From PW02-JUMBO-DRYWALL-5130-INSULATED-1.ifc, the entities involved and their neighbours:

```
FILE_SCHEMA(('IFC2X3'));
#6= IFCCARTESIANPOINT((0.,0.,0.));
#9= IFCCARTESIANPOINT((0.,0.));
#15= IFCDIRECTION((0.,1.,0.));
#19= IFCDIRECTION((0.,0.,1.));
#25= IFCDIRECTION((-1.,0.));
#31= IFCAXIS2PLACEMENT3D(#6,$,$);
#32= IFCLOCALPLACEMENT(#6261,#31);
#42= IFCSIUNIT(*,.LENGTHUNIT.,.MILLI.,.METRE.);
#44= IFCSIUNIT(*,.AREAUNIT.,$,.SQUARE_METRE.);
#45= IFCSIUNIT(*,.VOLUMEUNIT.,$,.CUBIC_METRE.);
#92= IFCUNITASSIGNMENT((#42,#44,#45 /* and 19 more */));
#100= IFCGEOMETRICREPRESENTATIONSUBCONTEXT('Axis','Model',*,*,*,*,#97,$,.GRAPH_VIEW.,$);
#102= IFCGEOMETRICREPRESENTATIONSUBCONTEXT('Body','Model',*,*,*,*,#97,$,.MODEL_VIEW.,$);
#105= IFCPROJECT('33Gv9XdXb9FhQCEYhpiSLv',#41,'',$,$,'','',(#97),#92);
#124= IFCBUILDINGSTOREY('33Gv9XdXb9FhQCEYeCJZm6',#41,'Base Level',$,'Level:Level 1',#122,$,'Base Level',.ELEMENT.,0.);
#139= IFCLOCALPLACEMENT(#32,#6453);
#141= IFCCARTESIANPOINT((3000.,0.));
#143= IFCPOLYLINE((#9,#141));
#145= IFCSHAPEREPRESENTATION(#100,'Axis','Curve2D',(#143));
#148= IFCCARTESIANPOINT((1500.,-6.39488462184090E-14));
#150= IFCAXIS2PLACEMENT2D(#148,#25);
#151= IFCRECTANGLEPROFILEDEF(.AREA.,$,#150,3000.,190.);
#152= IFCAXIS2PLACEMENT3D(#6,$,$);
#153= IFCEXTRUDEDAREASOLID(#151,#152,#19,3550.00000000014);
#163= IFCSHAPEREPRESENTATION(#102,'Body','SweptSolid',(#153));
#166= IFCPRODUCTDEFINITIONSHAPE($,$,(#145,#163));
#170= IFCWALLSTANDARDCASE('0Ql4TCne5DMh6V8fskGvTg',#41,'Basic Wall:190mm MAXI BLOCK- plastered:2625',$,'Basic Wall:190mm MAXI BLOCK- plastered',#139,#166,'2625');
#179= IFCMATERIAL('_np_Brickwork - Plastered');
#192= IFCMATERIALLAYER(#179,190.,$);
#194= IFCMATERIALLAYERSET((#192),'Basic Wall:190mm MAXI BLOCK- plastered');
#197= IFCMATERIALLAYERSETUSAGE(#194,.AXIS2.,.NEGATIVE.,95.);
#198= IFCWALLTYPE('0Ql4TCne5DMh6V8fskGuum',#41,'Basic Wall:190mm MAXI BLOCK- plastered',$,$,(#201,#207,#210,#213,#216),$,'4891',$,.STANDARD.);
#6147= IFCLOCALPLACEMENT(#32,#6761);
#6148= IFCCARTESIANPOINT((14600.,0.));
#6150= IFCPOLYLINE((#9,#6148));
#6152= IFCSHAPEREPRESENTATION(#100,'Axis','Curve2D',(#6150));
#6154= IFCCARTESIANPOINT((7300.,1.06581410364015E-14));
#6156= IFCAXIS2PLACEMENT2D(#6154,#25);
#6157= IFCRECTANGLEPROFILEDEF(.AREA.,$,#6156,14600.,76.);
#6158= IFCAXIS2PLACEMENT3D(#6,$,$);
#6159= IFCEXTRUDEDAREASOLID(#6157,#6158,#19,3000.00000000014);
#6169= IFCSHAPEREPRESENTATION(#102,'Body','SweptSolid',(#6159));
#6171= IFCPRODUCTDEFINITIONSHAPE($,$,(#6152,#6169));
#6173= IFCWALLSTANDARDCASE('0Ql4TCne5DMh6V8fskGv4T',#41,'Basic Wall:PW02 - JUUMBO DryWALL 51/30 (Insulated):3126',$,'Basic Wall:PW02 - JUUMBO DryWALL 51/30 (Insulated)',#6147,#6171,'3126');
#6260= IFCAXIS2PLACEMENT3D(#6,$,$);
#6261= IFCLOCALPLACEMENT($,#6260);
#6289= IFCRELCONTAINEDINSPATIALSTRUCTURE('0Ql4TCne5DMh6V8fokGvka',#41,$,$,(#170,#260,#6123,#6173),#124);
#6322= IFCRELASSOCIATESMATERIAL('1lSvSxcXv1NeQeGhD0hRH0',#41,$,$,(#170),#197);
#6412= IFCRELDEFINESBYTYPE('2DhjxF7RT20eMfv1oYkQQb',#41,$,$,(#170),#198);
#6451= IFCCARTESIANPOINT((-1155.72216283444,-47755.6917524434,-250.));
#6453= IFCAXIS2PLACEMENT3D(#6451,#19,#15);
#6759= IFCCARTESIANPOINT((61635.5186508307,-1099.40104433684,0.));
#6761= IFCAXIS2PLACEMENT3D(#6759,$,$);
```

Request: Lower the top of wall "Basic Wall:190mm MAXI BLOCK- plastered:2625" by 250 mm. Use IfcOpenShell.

```python
import ifcopenshell
import ifcopenshell.geom
import ifcopenshell.util.representation
import ifcopenshell.util.shape

model = ifcopenshell.open("PW02-JUMBO-DRYWALL-5130-INSULATED-1.ifc")
settings = ifcopenshell.geom.settings()


def volume(element):
    """Net volume in cubic metres, openings subtracted."""
    shape = ifcopenshell.geom.create_shape(settings, element)
    return ifcopenshell.util.shape.get_volume(shape.geometry)


wall = model.by_id(170)
before = volume(wall)

body = ifcopenshell.util.representation.get_representation(wall, "Model", "Body")
solid = body.Items[0]
old_height = solid.Depth
solid.Depth -= 250.0
after = volume(wall)

print(f"height {old_height:g} -> {solid.Depth:g}, volume {before:.3f} -> {after:.3f} m3")

model.write("PW02-JUMBO-DRYWALL-5130-INSULATED-1_v2.ifc")
```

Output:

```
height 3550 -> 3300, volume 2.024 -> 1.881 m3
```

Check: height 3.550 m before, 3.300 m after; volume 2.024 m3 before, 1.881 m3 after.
